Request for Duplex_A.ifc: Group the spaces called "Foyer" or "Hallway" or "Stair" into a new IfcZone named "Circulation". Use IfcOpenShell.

First a look at what the model holds.

```python
import ifcopenshell

model = ifcopenshell.open("Duplex_A.ifc")
print(model.schema)
seen = {}
for space in model.by_type("IfcSpace"):
    seen[space.LongName] = seen.get(space.LongName, 0) + 1
for name, count in sorted(seen.items(), key=str):
    print(count, "x", name)
print("zones:", [z.Name for z in model.by_type("IfcZone")][:20])
```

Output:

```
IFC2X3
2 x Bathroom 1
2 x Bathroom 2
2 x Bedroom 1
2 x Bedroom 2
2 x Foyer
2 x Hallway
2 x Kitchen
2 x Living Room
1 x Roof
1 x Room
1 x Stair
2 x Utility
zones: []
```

```python
import ifcopenshell
import ifcopenshell.api.group
import ifcopenshell.api.root

model = ifcopenshell.open("Duplex_A.ifc")

names = {"Foyer", "Hallway", "Stair"}
spaces = [s for s in model.by_type("IfcSpace") if s.LongName in names]

zone = ifcopenshell.api.root.create_entity(model, ifc_class="IfcZone", name="Circulation")
ifcopenshell.api.group.assign_group(model, products=spaces, group=zone)
print(len(spaces), "spaces in", zone.Name)

model.write("Duplex_A-out.ifc")
```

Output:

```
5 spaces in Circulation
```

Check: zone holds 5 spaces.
